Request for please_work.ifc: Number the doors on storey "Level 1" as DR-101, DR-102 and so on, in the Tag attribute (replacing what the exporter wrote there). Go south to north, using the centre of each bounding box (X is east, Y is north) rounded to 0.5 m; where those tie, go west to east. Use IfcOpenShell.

First a look at what the model holds.

```python
import ifcopenshell
import ifcopenshell.util.element
import ifcopenshell.util.placement

model = ifcopenshell.open("please_work.ifc")
print(model.schema)
storey = next(s for s in model.by_type("IfcBuildingStorey") if s.Name == "Level 1")
doors = [e for e in ifcopenshell.util.element.get_decomposition(storey) if e.is_a("IfcDoor")]
for e in sorted(doors, key=lambda e: e.id()):
    origin = ifcopenshell.util.placement.get_local_placement(e.ObjectPlacement)[:3, 3]
    print(e.id(), e.Tag, e.Name, origin.round(2) + 0.0, sep=" | ")
```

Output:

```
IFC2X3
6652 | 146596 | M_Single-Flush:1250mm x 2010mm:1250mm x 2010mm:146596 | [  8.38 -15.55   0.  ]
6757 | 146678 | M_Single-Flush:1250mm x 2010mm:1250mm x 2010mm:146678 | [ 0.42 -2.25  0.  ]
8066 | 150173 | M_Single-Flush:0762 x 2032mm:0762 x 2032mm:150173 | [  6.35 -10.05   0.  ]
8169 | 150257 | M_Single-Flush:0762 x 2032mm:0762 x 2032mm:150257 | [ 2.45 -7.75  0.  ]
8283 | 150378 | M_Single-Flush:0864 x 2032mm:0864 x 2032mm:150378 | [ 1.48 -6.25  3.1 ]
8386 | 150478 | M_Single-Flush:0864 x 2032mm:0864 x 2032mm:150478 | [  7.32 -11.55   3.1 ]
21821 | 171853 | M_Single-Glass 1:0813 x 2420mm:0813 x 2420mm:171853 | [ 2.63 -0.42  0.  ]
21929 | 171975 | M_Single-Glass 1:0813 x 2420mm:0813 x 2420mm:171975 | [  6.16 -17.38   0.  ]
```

```python
import ifcopenshell
import ifcopenshell.geom
import ifcopenshell.util.element
import ifcopenshell.util.shape

model = ifcopenshell.open("please_work.ifc")
settings = ifcopenshell.geom.settings()
settings.set("use-world-coords", True)


def centre(element):
    shape = ifcopenshell.geom.create_shape(settings, element)
    return ifcopenshell.util.shape.get_bbox_centroid(shape.geometry)


storey = next(s for s in model.by_type("IfcBuildingStorey") if s.Name == "Level 1")
doors = [e for e in ifcopenshell.util.element.get_decomposition(storey) if e.is_a("IfcDoor")]

# Insertion points can sit at a corner or the storey origin, so sort by the geometry (in metres).
centres = {e: centre(e) for e in doors}
doors.sort(key=lambda e: (round(centres[e][1] / 0.5), centres[e][0]))

for i, e in enumerate(doors, start=1):
    number = f"DR-1{i:02d}"
    e.Tag = number
    print(e.id(), number)

model.write("please_work_updated.ifc")
```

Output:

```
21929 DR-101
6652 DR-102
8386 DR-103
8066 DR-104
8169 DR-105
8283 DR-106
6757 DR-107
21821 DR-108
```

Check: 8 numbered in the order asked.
